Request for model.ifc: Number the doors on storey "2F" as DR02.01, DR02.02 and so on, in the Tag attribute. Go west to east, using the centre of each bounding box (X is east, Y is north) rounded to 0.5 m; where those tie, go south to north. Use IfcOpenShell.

First a look at what the model holds.

```python
import ifcopenshell
import ifcopenshell.util.element
import ifcopenshell.util.placement

model = ifcopenshell.open("model.ifc")
print(model.schema)
storey = next(s for s in model.by_type("IfcBuildingStorey") if s.Name == "2F")
doors = [e for e in ifcopenshell.util.element.get_decomposition(storey) if e.is_a("IfcDoor")]
for e in sorted(doors, key=lambda e: e.id()):
    origin = ifcopenshell.util.placement.get_local_placement(e.ObjectPlacement)[:3, 3]
    print(e.id(), e.Tag, e.Name, origin.round(2) + 0.0, sep=" | ")
```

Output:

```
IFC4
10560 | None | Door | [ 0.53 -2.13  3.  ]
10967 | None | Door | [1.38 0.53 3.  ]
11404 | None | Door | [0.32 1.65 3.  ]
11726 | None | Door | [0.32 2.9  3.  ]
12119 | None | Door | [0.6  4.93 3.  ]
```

```python
import ifcopenshell
import ifcopenshell.geom
import ifcopenshell.util.element
import ifcopenshell.util.shape

model = ifcopenshell.open("model.ifc")
settings = ifcopenshell.geom.settings()
settings.set("use-world-coords", True)


def centre(element):
    shape = ifcopenshell.geom.create_shape(settings, element)
    return ifcopenshell.util.shape.get_bbox_centroid(shape.geometry)


storey = next(s for s in model.by_type("IfcBuildingStorey") if s.Name == "2F")
doors = [e for e in ifcopenshell.util.element.get_decomposition(storey) if e.is_a("IfcDoor")]

# Insertion points can sit at a corner or the storey origin, so sort by the geometry (in metres).
centres = {e: centre(e) for e in doors}
doors.sort(key=lambda e: (round(centres[e][0] / 0.5), centres[e][1]))

for i, e in enumerate(doors, start=1):
    number = f"DR02.{i:02d}"
    e.Tag = number
    print(e.id(), number)

model.write("model_v2.ifc")
```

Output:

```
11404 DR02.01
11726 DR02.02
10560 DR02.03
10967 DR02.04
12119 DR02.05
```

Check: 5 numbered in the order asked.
